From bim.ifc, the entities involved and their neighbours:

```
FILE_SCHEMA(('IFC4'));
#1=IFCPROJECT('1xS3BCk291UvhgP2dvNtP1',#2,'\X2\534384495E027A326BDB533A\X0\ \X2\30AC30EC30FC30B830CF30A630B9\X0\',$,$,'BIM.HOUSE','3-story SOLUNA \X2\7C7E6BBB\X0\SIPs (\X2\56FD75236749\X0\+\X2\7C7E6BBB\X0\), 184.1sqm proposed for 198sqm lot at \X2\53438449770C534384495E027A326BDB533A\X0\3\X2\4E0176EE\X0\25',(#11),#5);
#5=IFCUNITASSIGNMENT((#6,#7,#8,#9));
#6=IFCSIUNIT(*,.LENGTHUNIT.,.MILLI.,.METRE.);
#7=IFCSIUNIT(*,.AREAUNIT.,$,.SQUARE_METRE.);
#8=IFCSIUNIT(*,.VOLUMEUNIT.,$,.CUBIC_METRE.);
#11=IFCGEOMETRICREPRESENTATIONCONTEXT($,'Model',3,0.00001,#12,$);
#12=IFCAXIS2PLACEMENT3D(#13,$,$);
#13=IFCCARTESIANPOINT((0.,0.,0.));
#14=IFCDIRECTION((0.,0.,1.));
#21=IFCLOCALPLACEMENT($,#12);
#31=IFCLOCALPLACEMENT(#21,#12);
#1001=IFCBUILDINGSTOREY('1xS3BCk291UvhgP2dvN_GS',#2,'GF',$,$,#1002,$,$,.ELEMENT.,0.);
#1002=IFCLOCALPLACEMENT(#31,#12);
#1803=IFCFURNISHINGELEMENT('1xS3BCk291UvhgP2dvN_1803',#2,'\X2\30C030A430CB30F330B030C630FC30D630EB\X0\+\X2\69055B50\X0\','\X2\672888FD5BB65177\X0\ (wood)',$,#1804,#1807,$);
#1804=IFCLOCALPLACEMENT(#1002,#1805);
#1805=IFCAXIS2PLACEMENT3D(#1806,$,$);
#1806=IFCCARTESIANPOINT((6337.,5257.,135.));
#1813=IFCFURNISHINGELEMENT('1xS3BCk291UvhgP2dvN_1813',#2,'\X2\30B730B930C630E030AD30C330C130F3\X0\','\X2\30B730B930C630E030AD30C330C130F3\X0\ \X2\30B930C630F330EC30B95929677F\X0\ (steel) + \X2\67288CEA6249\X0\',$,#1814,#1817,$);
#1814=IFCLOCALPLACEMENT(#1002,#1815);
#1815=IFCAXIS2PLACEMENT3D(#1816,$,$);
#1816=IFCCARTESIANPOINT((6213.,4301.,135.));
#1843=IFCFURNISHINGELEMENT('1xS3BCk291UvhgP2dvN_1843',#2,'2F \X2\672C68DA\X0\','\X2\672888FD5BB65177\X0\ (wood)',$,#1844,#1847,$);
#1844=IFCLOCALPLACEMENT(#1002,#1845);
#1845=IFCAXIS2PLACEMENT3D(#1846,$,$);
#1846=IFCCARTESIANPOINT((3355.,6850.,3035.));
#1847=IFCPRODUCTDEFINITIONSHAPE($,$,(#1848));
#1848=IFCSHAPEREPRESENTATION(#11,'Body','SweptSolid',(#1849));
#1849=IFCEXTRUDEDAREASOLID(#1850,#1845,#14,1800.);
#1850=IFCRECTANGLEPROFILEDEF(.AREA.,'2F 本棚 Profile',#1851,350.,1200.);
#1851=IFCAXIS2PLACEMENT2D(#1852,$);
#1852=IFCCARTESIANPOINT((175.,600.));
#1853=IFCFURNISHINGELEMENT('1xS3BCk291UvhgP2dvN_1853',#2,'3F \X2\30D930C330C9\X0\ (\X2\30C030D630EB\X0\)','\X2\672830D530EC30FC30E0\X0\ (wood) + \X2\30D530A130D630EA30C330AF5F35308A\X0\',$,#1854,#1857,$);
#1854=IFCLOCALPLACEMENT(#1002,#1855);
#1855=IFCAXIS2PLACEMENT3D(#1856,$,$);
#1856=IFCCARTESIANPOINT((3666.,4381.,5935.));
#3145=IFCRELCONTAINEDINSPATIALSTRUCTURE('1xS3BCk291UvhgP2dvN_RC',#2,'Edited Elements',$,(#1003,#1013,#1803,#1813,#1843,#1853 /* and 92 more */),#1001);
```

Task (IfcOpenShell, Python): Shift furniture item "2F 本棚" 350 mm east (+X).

```python
import ifcopenshell
import ifcopenshell.api.geometry
import ifcopenshell.util.placement
import ifcopenshell.util.unit

model = ifcopenshell.open("bim.ifc")
unit_scale = ifcopenshell.util.unit.calculate_unit_scale(model)

item = model.by_guid("1xS3BCk291UvhgP2dvN_1843")
matrix = ifcopenshell.util.placement.get_local_placement(item.ObjectPlacement)
matrix[0, 3] += 0.35 / unit_scale
ifcopenshell.api.geometry.edit_object_placement(model, product=item, matrix=matrix, is_si=False)

print(ifcopenshell.util.placement.get_local_placement(item.ObjectPlacement).round(3) + 0.0)

model.write("bim_edited.ifc")
```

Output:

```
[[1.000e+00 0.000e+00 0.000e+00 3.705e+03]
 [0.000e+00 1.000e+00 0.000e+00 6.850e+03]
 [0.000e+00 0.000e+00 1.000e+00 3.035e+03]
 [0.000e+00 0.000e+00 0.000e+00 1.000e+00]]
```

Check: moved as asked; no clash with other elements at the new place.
